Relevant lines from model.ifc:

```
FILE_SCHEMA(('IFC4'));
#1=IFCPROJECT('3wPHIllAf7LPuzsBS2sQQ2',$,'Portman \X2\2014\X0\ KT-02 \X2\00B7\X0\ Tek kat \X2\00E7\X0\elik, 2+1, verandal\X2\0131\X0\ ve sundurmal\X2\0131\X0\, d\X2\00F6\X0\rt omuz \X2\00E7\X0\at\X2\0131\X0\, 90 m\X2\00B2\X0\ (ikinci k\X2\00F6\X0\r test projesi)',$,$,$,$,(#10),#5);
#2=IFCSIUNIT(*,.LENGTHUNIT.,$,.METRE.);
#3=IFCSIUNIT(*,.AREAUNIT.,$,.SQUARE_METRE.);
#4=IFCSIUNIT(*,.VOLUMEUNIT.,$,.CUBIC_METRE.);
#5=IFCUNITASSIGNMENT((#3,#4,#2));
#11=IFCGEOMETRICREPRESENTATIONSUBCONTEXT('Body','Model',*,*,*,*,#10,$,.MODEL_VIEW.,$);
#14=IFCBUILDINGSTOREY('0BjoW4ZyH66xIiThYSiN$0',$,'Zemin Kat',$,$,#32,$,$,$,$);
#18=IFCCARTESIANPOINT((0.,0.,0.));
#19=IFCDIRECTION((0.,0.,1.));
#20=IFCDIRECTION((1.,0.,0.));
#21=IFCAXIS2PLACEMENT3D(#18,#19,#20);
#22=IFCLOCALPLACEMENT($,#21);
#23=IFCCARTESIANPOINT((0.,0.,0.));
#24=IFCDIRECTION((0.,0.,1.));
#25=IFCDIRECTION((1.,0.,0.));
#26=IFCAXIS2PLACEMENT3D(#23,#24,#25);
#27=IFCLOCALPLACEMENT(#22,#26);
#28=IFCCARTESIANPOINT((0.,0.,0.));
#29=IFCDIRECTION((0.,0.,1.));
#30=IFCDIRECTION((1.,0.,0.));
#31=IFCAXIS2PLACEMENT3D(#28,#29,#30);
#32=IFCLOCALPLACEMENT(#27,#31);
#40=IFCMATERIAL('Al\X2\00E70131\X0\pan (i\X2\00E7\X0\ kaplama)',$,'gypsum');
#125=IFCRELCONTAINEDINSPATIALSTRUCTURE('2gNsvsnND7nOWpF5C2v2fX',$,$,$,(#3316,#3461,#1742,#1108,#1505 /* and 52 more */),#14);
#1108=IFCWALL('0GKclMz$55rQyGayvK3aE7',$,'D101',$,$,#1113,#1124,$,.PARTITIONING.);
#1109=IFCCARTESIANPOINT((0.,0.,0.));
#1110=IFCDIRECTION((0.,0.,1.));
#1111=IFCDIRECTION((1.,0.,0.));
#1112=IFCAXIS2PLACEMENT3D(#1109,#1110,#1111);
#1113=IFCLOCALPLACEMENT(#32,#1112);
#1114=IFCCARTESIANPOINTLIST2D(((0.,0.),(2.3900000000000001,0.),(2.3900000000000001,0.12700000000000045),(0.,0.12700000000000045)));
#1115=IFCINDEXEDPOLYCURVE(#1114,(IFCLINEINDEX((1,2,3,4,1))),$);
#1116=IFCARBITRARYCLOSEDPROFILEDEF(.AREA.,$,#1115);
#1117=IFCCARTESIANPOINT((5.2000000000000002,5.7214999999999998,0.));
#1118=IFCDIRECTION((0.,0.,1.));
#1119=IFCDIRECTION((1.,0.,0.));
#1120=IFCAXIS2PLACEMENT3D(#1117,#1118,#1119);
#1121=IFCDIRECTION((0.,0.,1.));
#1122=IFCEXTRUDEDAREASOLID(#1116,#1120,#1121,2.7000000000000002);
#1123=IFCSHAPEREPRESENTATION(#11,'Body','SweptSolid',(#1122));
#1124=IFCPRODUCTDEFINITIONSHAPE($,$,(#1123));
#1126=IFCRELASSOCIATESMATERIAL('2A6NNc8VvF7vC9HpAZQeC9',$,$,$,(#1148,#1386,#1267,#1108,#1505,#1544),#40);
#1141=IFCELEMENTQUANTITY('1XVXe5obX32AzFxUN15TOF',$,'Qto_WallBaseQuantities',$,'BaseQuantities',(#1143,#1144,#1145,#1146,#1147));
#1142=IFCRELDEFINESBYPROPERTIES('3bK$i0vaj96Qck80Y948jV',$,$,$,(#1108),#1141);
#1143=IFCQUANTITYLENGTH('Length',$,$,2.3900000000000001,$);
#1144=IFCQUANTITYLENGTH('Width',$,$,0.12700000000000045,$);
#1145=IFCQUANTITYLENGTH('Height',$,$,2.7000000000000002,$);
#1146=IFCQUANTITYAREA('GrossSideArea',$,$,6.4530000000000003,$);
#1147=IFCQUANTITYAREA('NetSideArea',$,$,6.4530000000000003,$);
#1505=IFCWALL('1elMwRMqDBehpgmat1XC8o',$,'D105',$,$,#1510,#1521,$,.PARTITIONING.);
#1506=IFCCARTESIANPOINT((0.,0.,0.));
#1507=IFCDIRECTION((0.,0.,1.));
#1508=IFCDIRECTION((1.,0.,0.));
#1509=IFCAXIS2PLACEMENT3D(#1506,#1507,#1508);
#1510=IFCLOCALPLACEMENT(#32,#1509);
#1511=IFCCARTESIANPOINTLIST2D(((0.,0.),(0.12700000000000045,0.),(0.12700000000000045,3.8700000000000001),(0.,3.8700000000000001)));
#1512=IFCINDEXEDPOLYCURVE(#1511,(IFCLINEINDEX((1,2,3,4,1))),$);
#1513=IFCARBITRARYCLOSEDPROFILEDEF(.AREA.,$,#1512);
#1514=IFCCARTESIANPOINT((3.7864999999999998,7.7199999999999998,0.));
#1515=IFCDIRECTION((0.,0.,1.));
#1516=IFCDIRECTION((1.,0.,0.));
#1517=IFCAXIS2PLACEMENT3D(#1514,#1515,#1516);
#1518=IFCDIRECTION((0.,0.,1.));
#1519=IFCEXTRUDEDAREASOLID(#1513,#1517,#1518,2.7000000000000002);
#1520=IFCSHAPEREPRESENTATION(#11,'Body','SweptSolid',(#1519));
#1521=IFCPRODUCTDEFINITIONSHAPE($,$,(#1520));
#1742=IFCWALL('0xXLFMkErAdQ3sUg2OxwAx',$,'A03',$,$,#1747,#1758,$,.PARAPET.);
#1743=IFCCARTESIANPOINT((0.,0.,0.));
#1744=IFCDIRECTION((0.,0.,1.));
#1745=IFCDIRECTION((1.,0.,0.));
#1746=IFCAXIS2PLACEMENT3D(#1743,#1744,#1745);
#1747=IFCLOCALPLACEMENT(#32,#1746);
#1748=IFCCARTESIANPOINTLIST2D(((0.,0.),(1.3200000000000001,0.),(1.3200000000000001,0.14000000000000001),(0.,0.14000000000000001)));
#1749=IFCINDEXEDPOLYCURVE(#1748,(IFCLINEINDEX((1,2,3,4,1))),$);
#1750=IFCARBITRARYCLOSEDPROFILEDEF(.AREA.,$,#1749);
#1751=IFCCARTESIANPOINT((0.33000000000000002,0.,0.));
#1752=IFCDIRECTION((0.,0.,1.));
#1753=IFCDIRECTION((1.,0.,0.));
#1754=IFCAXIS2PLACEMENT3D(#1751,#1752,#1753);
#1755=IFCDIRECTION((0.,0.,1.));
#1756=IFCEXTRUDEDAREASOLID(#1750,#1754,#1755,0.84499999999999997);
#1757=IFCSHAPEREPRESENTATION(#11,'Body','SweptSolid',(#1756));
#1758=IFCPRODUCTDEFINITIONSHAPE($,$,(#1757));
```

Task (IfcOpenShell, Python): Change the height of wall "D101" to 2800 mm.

```python
import ifcopenshell
import ifcopenshell.api.pset
import ifcopenshell.geom
import ifcopenshell.util.element
import ifcopenshell.util.representation
import ifcopenshell.util.shape
import ifcopenshell.util.unit

model = ifcopenshell.open("model.ifc")
unit_scale = ifcopenshell.util.unit.calculate_unit_scale(model)
area_scale = ifcopenshell.util.unit.calculate_unit_scale(model, "AREAUNIT")
settings = ifcopenshell.geom.settings()


def volume(element):
    """Net volume in cubic metres, openings subtracted."""
    shape = ifcopenshell.geom.create_shape(settings, element)
    return ifcopenshell.util.shape.get_volume(shape.geometry)


wall = model.by_guid("0GKclMz$55rQyGayvK3aE7")
before = volume(wall)

body = ifcopenshell.util.representation.get_representation(wall, "Model", "Body")
solid = body.Items[0]
old_height = solid.Depth
solid.Depth = 2.8
after = volume(wall)
thickness = 0.127  # wall thickness in metres

# Update the stored height, areas and volumes.
qto = model.by_id(ifcopenshell.util.element.get_pset(wall, "Qto_WallBaseQuantities", should_inherit=False)["id"])
ifcopenshell.api.pset.edit_qto(model, qto=qto, properties={
    "Height": solid.Depth,
    "GrossSideArea": ifcopenshell.util.element.get_pset(wall, "Qto_WallBaseQuantities", "GrossSideArea") * solid.Depth / old_height,
    "NetSideArea": after / thickness / area_scale,
})

print(f"height {old_height:g} -> {solid.Depth:g}, volume {before:.3f} -> {after:.3f} m3")

model.write("model_updated.ifc")
```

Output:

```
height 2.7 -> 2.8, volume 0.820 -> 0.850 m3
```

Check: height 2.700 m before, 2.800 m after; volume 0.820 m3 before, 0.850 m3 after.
